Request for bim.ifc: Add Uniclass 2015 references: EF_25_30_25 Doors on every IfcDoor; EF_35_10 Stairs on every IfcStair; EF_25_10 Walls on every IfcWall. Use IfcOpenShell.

First a look at what the model holds.

```python
import ifcopenshell

model = ifcopenshell.open("bim.ifc")
print(model.schema)
print("classifications:", [c.Name for c in model.by_type("IfcClassification")])
for ifc_class in ("IfcDoor", "IfcRoof", "IfcStair", "IfcWall", "IfcWindow"):
    print(ifc_class, len(model.by_type(ifc_class)))
```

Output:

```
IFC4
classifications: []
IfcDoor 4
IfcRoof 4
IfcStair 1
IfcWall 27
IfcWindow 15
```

```python
import ifcopenshell
import ifcopenshell.api.classification

model = ifcopenshell.open("bim.ifc")

system = ifcopenshell.api.classification.add_classification(model, classification="Uniclass 2015")

codes = {
    "IfcDoor": ("EF_25_30_25", "Doors"),
    "IfcStair": ("EF_35_10", "Stairs"),
    "IfcWall": ("EF_25_10", "Walls"),
}
for ifc_class, (code, name) in codes.items():
    products = model.by_type(ifc_class)
    ifcopenshell.api.classification.add_reference(
        model, products=products, classification=system, identification=code, name=name
    )
    print(code, len(products))

model.write("bim-out.ifc")
```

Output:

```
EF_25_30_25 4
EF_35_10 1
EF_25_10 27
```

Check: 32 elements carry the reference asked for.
